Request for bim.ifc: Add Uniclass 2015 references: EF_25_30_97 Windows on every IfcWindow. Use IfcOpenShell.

First a look at what the model holds.

```python
import ifcopenshell

model = ifcopenshell.open("bim.ifc")
print(model.schema)
print("classifications:", [c.Name for c in model.by_type("IfcClassification")])
for ifc_class in ("IfcDoor", "IfcRoof", "IfcStair", "IfcWall", "IfcWindow"):
    print(ifc_class, len(model.by_type(ifc_class)))
```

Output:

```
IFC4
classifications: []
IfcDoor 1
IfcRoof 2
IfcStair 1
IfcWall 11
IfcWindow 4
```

```python
import ifcopenshell
import ifcopenshell.api.classification

model = ifcopenshell.open("bim.ifc")

system = ifcopenshell.api.classification.add_classification(model, classification="Uniclass 2015")

codes = {
    "IfcWindow": ("EF_25_30_97", "Windows"),
}
for ifc_class, (code, name) in codes.items():
    products = model.by_type(ifc_class)
    ifcopenshell.api.classification.add_reference(
        model, products=products, classification=system, identification=code, name=name
    )
    print(code, len(products))

model.write("bim_v2.ifc")
```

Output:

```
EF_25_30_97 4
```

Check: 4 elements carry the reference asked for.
